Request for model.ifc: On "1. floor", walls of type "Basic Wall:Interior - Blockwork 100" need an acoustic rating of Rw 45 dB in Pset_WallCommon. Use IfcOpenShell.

First a look at what the model holds.

```python
import ifcopenshell
import ifcopenshell.util.element

model = ifcopenshell.open("model.ifc")
print(model.schema)
storey = next(s for s in model.by_type("IfcBuildingStorey") if s.Name == "1. floor")
walls = [e for e in ifcopenshell.util.element.get_decomposition(storey) if e.is_a("IfcWall")]
seen = {}
for e in walls:
    element_type = ifcopenshell.util.element.get_type(e)
    key = (element_type.Name if element_type != e and element_type else None, ifcopenshell.util.element.get_pset(e, "Pset_WallCommon", "AcousticRating"))
    seen[key] = seen.get(key, 0) + 1
for (name, value), count in sorted(seen.items(), key=str):
    print(count, "x", name, "|", value)
```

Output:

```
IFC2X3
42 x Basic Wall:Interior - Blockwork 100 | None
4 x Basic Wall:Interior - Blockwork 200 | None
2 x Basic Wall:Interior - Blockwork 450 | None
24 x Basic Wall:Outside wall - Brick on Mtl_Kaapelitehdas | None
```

```python
import ifcopenshell
import ifcopenshell.api.pset
import ifcopenshell.util.element

model = ifcopenshell.open("model.ifc")

storey = next(s for s in model.by_type("IfcBuildingStorey") if s.Name == "1. floor")
walls = [e for e in ifcopenshell.util.element.get_decomposition(storey) if e.is_a("IfcWall")]

count = 0
for e in walls:
    element_type = ifcopenshell.util.element.get_type(e)
    if element_type in (None, e) or element_type.Name != "Basic Wall:Interior - Blockwork 100":
        continue
    # add_pset returns the element's existing set when there is one.
    pset = ifcopenshell.api.pset.add_pset(model, product=e, name="Pset_WallCommon")
    ifcopenshell.api.pset.edit_pset(model, pset=pset, properties={"AcousticRating": "Rw 45 dB"})
    count += 1

print(count, "walls updated")

model.write("model-out.ifc")
```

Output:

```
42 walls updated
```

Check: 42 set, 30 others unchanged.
